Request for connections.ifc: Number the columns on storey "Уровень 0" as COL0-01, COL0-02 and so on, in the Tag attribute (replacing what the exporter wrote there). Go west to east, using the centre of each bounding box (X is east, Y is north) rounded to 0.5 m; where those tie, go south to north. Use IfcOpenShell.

First a look at what the model holds.

```python
import ifcopenshell
import ifcopenshell.util.element
import ifcopenshell.util.placement

model = ifcopenshell.open("connections.ifc")
print(model.schema)
storey = next(s for s in model.by_type("IfcBuildingStorey") if s.Name == "Уровень 0")
columns = [e for e in ifcopenshell.util.element.get_decomposition(storey) if e.is_a("IfcColumn")]
for e in sorted(columns, key=lambda e: e.id()):
    origin = ifcopenshell.util.placement.get_local_placement(e.ObjectPlacement)[:3, 3]
    print(e.id(), e.Tag, e.Name, origin.round(2) + 0.0, sep=" | ")
```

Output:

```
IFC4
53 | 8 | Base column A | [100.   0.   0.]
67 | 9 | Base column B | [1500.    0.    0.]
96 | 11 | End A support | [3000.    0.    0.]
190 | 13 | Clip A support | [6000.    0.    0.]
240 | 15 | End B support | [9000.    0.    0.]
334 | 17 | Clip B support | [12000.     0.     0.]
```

```python
import ifcopenshell
import ifcopenshell.geom
import ifcopenshell.util.element
import ifcopenshell.util.shape

model = ifcopenshell.open("connections.ifc")
settings = ifcopenshell.geom.settings()
settings.set("use-world-coords", True)


def centre(element):
    shape = ifcopenshell.geom.create_shape(settings, element)
    return ifcopenshell.util.shape.get_bbox_centroid(shape.geometry)


storey = next(s for s in model.by_type("IfcBuildingStorey") if s.Name == "Уровень 0")
columns = [e for e in ifcopenshell.util.element.get_decomposition(storey) if e.is_a("IfcColumn")]

# Insertion points can sit at a corner or the storey origin, so sort by the geometry (in metres).
centres = {e: centre(e) for e in columns}
columns.sort(key=lambda e: (round(centres[e][0] / 0.5), centres[e][1]))

for i, e in enumerate(columns, start=1):
    number = f"COL0-{i:02d}"
    e.Tag = number
    print(e.id(), number)

model.write("connections_edited.ifc")
```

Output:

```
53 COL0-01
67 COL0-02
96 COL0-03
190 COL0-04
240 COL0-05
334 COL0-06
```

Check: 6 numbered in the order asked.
